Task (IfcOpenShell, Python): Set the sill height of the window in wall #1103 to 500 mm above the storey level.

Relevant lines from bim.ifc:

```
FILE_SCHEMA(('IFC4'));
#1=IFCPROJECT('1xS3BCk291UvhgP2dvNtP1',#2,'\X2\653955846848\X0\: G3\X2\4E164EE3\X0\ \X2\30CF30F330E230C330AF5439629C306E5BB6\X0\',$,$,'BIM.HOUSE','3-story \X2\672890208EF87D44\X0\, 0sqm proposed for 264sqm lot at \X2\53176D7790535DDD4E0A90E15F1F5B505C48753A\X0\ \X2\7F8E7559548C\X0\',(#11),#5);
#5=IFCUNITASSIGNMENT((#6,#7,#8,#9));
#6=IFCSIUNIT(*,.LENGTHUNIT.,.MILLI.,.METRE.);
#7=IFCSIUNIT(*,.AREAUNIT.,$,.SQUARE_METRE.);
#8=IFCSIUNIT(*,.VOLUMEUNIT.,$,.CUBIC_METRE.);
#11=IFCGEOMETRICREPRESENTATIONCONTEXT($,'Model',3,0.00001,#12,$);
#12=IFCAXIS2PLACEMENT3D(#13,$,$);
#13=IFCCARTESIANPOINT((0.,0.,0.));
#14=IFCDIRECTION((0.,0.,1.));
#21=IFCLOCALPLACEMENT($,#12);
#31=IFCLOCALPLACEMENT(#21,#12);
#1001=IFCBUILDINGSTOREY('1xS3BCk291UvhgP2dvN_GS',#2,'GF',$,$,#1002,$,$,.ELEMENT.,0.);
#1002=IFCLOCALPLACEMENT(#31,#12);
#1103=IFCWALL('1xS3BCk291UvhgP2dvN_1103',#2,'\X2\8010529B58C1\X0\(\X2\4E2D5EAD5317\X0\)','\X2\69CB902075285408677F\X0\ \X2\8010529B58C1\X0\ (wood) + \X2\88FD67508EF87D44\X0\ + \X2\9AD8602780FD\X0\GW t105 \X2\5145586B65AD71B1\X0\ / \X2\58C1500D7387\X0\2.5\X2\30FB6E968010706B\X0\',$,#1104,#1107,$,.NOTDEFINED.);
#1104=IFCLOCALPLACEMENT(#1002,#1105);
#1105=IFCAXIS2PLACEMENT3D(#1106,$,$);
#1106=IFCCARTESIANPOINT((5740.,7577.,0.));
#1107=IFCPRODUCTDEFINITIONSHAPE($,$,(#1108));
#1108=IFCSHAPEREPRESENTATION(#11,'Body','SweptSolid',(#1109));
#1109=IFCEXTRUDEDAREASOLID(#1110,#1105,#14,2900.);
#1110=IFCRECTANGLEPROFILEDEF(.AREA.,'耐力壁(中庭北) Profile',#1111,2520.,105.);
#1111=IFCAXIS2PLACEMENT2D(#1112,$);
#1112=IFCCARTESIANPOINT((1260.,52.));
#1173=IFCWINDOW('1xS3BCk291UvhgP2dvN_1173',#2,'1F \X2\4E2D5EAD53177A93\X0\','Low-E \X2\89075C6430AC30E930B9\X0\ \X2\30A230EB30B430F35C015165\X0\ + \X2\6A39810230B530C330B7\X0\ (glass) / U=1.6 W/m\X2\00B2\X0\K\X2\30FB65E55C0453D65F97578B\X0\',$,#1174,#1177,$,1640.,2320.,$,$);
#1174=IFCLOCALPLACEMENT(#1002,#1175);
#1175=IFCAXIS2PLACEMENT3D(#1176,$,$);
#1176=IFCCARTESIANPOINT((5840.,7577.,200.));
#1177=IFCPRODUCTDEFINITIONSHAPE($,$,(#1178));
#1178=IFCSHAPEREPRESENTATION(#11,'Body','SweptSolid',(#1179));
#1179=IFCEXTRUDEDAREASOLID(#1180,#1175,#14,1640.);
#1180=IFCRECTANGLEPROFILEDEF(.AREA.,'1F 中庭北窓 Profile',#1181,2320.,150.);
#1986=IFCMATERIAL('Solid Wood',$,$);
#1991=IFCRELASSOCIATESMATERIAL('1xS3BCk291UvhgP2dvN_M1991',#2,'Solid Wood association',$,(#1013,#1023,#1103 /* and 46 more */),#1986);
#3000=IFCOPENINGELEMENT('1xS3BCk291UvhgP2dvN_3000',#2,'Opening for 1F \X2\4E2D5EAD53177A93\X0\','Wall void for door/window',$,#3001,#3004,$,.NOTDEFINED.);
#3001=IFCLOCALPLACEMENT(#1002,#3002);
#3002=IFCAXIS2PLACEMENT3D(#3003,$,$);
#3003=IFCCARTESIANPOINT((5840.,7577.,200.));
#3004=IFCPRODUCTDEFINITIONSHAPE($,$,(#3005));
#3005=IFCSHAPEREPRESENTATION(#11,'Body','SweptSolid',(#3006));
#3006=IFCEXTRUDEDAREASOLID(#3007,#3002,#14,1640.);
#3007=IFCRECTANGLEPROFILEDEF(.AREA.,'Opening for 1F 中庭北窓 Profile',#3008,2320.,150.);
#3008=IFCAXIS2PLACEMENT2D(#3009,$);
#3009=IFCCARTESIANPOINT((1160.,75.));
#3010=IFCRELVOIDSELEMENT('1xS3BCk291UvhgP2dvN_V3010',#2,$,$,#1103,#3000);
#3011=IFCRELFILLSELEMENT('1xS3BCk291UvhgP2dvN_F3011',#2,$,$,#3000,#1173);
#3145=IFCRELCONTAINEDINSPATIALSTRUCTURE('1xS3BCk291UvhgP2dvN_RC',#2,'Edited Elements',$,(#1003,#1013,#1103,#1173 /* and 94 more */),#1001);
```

```python
import numpy as np
import ifcopenshell
import ifcopenshell.api.geometry
import ifcopenshell.geom
import ifcopenshell.util.element
import ifcopenshell.util.placement
import ifcopenshell.util.shape
import ifcopenshell.util.unit

model = ifcopenshell.open("bim.ifc")
unit_scale = ifcopenshell.util.unit.calculate_unit_scale(model)

window = model.by_id(1173)
opening = window.FillsVoids[0].RelatingOpeningElement
storey = ifcopenshell.util.element.get_container(window, ifc_class="IfcBuildingStorey")
level = ifcopenshell.util.placement.get_local_placement(storey.ObjectPlacement)[2, 3]

# The opening's origin need not be at the sill, so measure its lowest point.
shape = ifcopenshell.geom.create_shape(ifcopenshell.geom.settings(), opening)
bottom = ifcopenshell.util.shape.get_shape_bottom_elevation(shape, shape.geometry) / unit_scale
dz = level + 0.5 / unit_scale - bottom

shift = np.array([0.0, 0.0, dz])
# The window is not placed relative to its opening, so move both.
for product in (opening, window):
    matrix = ifcopenshell.util.placement.get_local_placement(product.ObjectPlacement)
    matrix[:3, 3] += shift
    ifcopenshell.api.geometry.edit_object_placement(model, product=product, matrix=matrix, is_si=False)

print(f"moved by {dz * unit_scale:+.3f} m")

model.write("bim-out.ifc")
```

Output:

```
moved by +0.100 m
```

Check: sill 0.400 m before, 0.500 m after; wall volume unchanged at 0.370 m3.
